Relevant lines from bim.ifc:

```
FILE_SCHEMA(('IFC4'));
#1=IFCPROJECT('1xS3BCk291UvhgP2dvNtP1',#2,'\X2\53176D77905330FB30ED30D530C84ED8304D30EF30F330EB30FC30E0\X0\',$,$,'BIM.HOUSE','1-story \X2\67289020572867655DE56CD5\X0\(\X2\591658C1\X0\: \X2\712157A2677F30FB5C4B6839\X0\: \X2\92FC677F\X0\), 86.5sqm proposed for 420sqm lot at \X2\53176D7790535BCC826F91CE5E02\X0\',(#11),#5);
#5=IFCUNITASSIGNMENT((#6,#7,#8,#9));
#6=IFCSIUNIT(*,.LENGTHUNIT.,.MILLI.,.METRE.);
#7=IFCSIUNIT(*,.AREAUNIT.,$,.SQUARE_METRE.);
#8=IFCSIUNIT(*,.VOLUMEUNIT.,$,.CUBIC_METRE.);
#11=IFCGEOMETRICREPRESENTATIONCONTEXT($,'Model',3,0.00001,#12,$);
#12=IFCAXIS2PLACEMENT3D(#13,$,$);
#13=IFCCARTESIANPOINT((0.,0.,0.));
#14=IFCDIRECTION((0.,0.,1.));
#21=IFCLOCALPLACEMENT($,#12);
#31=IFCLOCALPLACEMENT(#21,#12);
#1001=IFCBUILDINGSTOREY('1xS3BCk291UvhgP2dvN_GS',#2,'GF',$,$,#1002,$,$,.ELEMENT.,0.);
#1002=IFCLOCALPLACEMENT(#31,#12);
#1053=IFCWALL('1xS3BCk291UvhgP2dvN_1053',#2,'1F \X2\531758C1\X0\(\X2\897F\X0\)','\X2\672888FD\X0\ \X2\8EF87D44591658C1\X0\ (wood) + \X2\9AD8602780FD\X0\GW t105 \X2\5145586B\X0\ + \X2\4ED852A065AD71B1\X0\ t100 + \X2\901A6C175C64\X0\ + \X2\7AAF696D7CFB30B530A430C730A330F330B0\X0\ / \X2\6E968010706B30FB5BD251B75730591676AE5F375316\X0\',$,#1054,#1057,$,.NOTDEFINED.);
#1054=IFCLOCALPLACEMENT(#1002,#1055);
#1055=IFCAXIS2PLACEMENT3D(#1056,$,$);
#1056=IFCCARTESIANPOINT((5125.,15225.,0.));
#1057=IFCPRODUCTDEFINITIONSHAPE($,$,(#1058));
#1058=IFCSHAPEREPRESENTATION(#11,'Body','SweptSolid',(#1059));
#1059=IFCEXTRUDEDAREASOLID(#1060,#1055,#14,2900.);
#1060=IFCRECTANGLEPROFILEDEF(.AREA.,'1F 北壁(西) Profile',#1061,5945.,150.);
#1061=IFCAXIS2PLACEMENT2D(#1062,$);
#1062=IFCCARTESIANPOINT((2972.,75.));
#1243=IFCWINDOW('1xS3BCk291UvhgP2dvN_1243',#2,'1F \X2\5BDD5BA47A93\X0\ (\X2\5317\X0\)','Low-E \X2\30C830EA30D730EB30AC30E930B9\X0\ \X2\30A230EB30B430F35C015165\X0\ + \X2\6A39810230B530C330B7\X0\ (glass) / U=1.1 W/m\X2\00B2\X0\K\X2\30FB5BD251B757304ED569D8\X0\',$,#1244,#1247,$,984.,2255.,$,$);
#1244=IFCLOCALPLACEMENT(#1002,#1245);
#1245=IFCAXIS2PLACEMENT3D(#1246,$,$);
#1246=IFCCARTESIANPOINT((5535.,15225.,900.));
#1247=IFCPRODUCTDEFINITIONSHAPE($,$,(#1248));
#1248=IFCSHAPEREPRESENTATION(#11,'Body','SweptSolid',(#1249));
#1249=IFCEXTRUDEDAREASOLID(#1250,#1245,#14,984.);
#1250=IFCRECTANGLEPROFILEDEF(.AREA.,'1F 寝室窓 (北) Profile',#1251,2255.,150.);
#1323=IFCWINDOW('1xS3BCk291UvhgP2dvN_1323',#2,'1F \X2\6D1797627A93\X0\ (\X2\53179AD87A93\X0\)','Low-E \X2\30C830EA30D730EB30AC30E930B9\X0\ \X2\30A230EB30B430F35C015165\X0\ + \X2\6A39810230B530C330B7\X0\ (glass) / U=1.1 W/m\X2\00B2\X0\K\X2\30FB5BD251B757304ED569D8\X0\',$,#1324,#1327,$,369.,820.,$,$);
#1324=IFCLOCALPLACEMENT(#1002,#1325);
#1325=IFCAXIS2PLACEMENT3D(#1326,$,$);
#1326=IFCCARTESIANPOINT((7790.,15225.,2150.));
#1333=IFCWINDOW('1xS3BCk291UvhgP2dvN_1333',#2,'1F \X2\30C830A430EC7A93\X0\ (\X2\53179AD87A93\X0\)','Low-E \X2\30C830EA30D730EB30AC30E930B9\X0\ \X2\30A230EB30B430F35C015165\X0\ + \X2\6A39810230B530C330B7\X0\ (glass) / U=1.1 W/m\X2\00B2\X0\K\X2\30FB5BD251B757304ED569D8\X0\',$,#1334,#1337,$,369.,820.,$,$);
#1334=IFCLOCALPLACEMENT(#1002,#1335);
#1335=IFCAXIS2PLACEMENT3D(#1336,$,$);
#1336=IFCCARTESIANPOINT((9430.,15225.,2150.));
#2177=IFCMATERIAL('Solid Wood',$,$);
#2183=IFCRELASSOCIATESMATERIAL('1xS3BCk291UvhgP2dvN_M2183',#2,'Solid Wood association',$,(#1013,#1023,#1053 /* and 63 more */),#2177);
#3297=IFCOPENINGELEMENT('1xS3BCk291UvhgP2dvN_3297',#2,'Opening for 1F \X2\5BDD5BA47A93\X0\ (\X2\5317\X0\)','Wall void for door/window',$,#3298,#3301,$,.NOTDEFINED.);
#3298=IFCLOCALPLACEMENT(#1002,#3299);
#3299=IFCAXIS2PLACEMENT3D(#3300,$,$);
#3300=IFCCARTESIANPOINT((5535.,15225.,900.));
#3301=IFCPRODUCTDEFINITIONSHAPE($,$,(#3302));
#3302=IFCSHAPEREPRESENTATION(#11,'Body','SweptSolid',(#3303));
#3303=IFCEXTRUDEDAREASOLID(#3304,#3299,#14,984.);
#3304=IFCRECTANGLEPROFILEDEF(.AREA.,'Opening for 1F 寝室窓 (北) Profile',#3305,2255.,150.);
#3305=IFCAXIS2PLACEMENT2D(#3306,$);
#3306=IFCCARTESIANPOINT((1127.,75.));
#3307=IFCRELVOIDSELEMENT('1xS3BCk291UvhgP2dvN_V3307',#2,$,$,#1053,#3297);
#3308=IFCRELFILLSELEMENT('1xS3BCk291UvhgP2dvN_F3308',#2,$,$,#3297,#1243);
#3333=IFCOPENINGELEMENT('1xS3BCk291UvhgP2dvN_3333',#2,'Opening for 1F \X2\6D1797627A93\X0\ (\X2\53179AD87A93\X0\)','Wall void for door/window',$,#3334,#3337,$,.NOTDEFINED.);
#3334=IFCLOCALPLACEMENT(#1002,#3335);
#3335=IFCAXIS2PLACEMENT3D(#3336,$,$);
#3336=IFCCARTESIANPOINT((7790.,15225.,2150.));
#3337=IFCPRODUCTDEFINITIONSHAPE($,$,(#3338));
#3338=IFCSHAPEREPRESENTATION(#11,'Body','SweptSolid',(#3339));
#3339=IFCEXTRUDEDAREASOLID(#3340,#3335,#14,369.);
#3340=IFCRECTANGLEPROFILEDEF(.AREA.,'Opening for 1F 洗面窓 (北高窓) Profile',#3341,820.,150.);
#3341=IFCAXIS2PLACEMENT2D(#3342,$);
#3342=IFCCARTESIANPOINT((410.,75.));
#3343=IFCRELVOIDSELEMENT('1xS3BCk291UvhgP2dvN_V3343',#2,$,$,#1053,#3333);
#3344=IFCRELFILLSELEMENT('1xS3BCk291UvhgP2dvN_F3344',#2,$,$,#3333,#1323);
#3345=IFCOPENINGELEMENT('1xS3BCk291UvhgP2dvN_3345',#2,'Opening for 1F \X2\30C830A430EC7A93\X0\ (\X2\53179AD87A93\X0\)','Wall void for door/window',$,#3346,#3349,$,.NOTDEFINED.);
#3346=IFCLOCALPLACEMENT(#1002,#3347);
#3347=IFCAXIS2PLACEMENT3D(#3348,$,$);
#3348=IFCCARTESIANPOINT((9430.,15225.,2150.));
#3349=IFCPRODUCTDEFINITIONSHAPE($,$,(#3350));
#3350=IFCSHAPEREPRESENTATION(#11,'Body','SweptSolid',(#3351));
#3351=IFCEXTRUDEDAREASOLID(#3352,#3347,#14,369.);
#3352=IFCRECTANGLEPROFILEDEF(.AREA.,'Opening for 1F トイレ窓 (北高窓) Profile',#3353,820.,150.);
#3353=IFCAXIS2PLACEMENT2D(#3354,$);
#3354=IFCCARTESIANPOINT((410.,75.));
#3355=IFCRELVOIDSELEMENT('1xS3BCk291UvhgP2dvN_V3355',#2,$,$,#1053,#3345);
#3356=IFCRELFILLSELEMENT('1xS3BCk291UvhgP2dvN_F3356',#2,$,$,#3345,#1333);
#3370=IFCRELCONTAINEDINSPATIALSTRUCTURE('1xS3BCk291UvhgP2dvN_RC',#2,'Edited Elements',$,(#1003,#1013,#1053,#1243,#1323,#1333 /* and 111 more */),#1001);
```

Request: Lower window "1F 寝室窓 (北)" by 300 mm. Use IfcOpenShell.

```python
import numpy as np
import ifcopenshell
import ifcopenshell.api.geometry
import ifcopenshell.util.placement
import ifcopenshell.util.unit

model = ifcopenshell.open("bim.ifc")
unit_scale = ifcopenshell.util.unit.calculate_unit_scale(model)

window = model.by_guid("1xS3BCk291UvhgP2dvN_1243")
opening = window.FillsVoids[0].RelatingOpeningElement
dz = -300.0

shift = np.array([0.0, 0.0, dz])
# The window is not placed relative to its opening, so move both.
for product in (opening, window):
    matrix = ifcopenshell.util.placement.get_local_placement(product.ObjectPlacement)
    matrix[:3, 3] += shift
    ifcopenshell.api.geometry.edit_object_placement(model, product=product, matrix=matrix, is_si=False)

print(f"moved by {dz * unit_scale:+.3f} m")

model.write("bim_updated.ifc")
```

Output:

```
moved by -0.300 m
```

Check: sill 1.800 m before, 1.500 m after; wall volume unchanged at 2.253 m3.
